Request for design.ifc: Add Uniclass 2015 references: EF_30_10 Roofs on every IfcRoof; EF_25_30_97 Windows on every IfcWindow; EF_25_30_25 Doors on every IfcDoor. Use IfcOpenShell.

First a look at what the model holds.

```python
import ifcopenshell

model = ifcopenshell.open("design.ifc")
print(model.schema)
print("classifications:", [c.Name for c in model.by_type("IfcClassification")])
for ifc_class in ("IfcDoor", "IfcRoof", "IfcStair", "IfcWall", "IfcWindow"):
    print(ifc_class, len(model.by_type(ifc_class)))
```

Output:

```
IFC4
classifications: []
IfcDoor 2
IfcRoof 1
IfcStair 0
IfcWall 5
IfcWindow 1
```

```python
import ifcopenshell
import ifcopenshell.api.classification

model = ifcopenshell.open("design.ifc")

system = ifcopenshell.api.classification.add_classification(model, classification="Uniclass 2015")

codes = {
    "IfcRoof": ("EF_30_10", "Roofs"),
    "IfcWindow": ("EF_25_30_97", "Windows"),
    "IfcDoor": ("EF_25_30_25", "Doors"),
}
for ifc_class, (code, name) in codes.items():
    products = model.by_type(ifc_class)
    ifcopenshell.api.classification.add_reference(
        model, products=products, classification=system, identification=code, name=name
    )
    print(code, len(products))

model.write("design_updated.ifc")
```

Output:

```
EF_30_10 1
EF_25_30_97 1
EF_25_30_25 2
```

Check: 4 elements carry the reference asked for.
